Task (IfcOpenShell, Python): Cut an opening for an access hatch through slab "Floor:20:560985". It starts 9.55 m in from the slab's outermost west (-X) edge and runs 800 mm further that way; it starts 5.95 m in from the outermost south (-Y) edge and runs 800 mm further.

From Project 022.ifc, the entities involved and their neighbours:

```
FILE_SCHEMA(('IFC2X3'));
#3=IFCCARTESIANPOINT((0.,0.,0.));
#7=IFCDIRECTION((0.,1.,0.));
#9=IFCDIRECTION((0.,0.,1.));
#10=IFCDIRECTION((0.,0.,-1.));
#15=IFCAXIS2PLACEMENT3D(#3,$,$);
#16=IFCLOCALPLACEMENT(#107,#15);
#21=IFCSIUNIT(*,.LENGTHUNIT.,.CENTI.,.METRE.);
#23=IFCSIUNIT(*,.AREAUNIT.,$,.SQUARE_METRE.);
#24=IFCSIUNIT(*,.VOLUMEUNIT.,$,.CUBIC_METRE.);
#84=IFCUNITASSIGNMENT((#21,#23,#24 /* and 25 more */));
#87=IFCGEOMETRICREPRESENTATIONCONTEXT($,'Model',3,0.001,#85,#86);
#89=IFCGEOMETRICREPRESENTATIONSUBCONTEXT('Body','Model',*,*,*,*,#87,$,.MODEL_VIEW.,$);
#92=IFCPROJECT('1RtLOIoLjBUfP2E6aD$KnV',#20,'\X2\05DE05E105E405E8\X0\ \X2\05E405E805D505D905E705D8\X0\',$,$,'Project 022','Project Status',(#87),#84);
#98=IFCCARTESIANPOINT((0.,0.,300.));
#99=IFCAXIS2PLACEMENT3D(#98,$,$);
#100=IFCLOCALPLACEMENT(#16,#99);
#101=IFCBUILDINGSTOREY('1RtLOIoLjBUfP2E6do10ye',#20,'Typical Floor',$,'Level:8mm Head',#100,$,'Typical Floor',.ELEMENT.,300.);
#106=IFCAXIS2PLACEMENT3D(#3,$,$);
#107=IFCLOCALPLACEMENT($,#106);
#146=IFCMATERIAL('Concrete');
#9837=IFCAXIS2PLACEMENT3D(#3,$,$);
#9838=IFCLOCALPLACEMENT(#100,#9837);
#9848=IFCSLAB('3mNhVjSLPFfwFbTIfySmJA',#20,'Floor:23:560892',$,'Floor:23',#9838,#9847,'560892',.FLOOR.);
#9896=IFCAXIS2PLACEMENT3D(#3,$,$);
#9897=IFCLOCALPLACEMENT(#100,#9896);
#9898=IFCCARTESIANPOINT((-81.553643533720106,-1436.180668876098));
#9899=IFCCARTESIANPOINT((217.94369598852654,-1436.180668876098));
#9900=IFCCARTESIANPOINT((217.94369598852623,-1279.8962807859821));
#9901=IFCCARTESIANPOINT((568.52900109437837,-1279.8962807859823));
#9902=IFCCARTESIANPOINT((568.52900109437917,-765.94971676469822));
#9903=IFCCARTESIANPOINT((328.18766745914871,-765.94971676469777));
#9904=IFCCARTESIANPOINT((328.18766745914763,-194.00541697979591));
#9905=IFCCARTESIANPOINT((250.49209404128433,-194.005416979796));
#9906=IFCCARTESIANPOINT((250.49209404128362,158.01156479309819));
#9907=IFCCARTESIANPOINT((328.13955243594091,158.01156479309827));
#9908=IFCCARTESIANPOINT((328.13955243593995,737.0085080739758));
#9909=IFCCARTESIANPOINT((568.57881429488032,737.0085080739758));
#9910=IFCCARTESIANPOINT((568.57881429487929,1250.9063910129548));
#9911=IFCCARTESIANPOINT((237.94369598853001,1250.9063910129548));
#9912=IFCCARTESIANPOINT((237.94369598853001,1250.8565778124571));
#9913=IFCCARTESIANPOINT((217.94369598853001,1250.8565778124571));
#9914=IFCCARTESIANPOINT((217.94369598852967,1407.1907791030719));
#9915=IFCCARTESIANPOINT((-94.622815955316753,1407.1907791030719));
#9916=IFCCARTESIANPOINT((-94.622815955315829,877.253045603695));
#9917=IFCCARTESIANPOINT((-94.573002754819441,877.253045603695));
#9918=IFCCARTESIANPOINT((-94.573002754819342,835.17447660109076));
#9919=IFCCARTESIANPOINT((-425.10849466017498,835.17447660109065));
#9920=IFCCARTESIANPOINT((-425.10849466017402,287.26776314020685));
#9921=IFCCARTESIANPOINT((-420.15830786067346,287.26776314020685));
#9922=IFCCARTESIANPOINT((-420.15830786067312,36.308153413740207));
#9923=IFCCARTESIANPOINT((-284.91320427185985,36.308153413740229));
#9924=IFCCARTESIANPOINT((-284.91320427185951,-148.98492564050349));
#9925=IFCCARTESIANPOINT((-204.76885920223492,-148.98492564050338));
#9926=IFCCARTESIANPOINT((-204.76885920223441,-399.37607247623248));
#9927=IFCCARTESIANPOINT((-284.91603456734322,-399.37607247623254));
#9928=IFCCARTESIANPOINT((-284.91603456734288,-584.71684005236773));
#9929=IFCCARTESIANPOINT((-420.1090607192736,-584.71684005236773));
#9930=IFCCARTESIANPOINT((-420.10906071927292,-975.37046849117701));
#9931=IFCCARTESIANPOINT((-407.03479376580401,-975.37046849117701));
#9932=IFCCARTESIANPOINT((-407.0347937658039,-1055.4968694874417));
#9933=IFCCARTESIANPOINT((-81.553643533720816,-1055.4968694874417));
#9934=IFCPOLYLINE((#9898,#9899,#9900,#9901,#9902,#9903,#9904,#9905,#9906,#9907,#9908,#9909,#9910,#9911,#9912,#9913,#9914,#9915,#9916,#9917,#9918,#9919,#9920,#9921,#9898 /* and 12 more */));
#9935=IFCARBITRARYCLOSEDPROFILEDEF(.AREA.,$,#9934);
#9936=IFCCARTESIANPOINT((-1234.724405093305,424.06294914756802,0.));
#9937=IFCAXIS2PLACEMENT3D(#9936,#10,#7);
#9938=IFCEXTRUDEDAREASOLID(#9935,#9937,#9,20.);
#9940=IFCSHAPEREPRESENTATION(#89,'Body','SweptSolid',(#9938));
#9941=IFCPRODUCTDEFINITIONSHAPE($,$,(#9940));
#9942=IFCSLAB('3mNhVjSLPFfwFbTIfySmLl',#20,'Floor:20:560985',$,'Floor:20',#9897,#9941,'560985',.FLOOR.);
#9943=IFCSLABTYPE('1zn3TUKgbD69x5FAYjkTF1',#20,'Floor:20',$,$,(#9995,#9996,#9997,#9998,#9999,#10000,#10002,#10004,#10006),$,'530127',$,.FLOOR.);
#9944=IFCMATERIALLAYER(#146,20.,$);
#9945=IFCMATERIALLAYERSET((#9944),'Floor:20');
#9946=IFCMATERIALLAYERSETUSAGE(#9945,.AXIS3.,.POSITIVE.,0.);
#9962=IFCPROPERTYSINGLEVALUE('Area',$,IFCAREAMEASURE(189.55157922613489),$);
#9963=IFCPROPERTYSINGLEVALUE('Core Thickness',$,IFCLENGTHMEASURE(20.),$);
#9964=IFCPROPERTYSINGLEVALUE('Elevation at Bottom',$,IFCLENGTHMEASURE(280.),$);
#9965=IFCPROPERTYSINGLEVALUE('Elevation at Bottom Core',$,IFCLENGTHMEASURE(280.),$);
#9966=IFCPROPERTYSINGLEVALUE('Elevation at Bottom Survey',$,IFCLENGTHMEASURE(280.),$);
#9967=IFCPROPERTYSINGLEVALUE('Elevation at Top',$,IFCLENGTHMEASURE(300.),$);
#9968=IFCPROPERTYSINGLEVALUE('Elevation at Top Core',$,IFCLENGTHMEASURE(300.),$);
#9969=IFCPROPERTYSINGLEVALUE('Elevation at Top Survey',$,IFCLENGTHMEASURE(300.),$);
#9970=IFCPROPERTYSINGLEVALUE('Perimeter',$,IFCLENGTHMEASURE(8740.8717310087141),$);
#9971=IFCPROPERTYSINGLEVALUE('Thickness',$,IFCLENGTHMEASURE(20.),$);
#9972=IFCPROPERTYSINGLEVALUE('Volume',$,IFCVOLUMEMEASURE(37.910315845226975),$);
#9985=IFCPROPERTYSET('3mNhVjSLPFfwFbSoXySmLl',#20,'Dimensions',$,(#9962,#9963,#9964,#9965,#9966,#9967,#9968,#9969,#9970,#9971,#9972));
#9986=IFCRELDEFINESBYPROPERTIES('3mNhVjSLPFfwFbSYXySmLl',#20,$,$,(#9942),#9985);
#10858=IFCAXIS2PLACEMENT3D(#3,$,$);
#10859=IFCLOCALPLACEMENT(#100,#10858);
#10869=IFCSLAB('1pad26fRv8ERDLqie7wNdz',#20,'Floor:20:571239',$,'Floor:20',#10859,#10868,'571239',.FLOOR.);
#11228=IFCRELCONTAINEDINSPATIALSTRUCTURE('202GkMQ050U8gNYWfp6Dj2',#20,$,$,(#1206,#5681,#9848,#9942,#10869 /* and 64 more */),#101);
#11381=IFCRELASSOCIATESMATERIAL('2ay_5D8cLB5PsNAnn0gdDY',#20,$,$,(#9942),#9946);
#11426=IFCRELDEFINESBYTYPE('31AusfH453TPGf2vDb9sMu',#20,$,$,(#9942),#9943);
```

```python
import numpy as np
import ifcopenshell
import ifcopenshell.api.feature
import ifcopenshell.api.geometry
import ifcopenshell.api.pset
import ifcopenshell.api.root
import ifcopenshell.geom
import ifcopenshell.util.element
import ifcopenshell.util.placement
import ifcopenshell.util.representation
import ifcopenshell.util.shape
import ifcopenshell.util.unit

model = ifcopenshell.open("Project 022.ifc")
unit_scale = ifcopenshell.util.unit.calculate_unit_scale(model)
area_scale = ifcopenshell.util.unit.calculate_unit_scale(model, "AREAUNIT")
volume_scale = ifcopenshell.util.unit.calculate_unit_scale(model, "VOLUMEUNIT")
settings = ifcopenshell.geom.settings()


def volume(element):
    """Net volume in cubic metres, openings subtracted."""
    shape = ifcopenshell.geom.create_shape(settings, element)
    return ifcopenshell.util.shape.get_volume(shape.geometry)


slab = model.by_guid("3mNhVjSLPFfwFbTIfySmLl")
before = volume(slab)

# Extent in the slab's own axes, in metres. The edges named are its -X and -Y sides.
slab_shape = ifcopenshell.geom.create_shape(settings, slab)
vertices = ifcopenshell.util.shape.get_vertices(slab_shape.geometry)
x_min, y_min, bottom = vertices.min(axis=0)
top = vertices[:, 2].max()

opening = ifcopenshell.api.root.create_entity(model, ifc_class="IfcOpeningElement", name="Access hatch opening")
context = ifcopenshell.util.representation.get_context(model, "Model", "Body", "MODEL_VIEW")
width, depth = 0.8, 0.8
outline = [(0.0, 0.0), (width, 0.0), (width, depth), (0.0, depth), (0.0, 0.0)]
# Overshoot both faces by 50 mm so the cut is clean.
shape = ifcopenshell.api.geometry.add_slab_representation(
    model, context=context, depth=top - bottom + 0.1, polyline=outline
)
ifcopenshell.api.geometry.assign_representation(model, product=opening, representation=shape)

matrix = ifcopenshell.util.placement.get_local_placement(slab.ObjectPlacement)
matrix[:, 3] = matrix @ np.append(np.array([x_min + 9.55, y_min + 5.95, bottom - 0.05]) / unit_scale, 1.0)
ifcopenshell.api.geometry.edit_object_placement(model, product=opening, matrix=matrix, is_si=False)
ifcopenshell.api.feature.add_feature(model, feature=opening, element=slab)

after = volume(slab)

# Update the slab's stored quantities.
pset = model.by_id(ifcopenshell.util.element.get_pset(slab, "Dimensions", should_inherit=False)["id"])
ifcopenshell.api.pset.edit_pset(model, pset=pset, properties={
    "Area": model.create_entity("IfcAreaMeasure", after / (top - bottom) / area_scale),
    "Volume": model.create_entity("IfcVolumeMeasure", after / volume_scale),
})

print(f"slab volume {before:.3f} -> {after:.3f} m3")

model.write("Project 022_rev.ifc")
```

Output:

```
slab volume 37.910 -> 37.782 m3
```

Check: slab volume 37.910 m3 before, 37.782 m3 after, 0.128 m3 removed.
